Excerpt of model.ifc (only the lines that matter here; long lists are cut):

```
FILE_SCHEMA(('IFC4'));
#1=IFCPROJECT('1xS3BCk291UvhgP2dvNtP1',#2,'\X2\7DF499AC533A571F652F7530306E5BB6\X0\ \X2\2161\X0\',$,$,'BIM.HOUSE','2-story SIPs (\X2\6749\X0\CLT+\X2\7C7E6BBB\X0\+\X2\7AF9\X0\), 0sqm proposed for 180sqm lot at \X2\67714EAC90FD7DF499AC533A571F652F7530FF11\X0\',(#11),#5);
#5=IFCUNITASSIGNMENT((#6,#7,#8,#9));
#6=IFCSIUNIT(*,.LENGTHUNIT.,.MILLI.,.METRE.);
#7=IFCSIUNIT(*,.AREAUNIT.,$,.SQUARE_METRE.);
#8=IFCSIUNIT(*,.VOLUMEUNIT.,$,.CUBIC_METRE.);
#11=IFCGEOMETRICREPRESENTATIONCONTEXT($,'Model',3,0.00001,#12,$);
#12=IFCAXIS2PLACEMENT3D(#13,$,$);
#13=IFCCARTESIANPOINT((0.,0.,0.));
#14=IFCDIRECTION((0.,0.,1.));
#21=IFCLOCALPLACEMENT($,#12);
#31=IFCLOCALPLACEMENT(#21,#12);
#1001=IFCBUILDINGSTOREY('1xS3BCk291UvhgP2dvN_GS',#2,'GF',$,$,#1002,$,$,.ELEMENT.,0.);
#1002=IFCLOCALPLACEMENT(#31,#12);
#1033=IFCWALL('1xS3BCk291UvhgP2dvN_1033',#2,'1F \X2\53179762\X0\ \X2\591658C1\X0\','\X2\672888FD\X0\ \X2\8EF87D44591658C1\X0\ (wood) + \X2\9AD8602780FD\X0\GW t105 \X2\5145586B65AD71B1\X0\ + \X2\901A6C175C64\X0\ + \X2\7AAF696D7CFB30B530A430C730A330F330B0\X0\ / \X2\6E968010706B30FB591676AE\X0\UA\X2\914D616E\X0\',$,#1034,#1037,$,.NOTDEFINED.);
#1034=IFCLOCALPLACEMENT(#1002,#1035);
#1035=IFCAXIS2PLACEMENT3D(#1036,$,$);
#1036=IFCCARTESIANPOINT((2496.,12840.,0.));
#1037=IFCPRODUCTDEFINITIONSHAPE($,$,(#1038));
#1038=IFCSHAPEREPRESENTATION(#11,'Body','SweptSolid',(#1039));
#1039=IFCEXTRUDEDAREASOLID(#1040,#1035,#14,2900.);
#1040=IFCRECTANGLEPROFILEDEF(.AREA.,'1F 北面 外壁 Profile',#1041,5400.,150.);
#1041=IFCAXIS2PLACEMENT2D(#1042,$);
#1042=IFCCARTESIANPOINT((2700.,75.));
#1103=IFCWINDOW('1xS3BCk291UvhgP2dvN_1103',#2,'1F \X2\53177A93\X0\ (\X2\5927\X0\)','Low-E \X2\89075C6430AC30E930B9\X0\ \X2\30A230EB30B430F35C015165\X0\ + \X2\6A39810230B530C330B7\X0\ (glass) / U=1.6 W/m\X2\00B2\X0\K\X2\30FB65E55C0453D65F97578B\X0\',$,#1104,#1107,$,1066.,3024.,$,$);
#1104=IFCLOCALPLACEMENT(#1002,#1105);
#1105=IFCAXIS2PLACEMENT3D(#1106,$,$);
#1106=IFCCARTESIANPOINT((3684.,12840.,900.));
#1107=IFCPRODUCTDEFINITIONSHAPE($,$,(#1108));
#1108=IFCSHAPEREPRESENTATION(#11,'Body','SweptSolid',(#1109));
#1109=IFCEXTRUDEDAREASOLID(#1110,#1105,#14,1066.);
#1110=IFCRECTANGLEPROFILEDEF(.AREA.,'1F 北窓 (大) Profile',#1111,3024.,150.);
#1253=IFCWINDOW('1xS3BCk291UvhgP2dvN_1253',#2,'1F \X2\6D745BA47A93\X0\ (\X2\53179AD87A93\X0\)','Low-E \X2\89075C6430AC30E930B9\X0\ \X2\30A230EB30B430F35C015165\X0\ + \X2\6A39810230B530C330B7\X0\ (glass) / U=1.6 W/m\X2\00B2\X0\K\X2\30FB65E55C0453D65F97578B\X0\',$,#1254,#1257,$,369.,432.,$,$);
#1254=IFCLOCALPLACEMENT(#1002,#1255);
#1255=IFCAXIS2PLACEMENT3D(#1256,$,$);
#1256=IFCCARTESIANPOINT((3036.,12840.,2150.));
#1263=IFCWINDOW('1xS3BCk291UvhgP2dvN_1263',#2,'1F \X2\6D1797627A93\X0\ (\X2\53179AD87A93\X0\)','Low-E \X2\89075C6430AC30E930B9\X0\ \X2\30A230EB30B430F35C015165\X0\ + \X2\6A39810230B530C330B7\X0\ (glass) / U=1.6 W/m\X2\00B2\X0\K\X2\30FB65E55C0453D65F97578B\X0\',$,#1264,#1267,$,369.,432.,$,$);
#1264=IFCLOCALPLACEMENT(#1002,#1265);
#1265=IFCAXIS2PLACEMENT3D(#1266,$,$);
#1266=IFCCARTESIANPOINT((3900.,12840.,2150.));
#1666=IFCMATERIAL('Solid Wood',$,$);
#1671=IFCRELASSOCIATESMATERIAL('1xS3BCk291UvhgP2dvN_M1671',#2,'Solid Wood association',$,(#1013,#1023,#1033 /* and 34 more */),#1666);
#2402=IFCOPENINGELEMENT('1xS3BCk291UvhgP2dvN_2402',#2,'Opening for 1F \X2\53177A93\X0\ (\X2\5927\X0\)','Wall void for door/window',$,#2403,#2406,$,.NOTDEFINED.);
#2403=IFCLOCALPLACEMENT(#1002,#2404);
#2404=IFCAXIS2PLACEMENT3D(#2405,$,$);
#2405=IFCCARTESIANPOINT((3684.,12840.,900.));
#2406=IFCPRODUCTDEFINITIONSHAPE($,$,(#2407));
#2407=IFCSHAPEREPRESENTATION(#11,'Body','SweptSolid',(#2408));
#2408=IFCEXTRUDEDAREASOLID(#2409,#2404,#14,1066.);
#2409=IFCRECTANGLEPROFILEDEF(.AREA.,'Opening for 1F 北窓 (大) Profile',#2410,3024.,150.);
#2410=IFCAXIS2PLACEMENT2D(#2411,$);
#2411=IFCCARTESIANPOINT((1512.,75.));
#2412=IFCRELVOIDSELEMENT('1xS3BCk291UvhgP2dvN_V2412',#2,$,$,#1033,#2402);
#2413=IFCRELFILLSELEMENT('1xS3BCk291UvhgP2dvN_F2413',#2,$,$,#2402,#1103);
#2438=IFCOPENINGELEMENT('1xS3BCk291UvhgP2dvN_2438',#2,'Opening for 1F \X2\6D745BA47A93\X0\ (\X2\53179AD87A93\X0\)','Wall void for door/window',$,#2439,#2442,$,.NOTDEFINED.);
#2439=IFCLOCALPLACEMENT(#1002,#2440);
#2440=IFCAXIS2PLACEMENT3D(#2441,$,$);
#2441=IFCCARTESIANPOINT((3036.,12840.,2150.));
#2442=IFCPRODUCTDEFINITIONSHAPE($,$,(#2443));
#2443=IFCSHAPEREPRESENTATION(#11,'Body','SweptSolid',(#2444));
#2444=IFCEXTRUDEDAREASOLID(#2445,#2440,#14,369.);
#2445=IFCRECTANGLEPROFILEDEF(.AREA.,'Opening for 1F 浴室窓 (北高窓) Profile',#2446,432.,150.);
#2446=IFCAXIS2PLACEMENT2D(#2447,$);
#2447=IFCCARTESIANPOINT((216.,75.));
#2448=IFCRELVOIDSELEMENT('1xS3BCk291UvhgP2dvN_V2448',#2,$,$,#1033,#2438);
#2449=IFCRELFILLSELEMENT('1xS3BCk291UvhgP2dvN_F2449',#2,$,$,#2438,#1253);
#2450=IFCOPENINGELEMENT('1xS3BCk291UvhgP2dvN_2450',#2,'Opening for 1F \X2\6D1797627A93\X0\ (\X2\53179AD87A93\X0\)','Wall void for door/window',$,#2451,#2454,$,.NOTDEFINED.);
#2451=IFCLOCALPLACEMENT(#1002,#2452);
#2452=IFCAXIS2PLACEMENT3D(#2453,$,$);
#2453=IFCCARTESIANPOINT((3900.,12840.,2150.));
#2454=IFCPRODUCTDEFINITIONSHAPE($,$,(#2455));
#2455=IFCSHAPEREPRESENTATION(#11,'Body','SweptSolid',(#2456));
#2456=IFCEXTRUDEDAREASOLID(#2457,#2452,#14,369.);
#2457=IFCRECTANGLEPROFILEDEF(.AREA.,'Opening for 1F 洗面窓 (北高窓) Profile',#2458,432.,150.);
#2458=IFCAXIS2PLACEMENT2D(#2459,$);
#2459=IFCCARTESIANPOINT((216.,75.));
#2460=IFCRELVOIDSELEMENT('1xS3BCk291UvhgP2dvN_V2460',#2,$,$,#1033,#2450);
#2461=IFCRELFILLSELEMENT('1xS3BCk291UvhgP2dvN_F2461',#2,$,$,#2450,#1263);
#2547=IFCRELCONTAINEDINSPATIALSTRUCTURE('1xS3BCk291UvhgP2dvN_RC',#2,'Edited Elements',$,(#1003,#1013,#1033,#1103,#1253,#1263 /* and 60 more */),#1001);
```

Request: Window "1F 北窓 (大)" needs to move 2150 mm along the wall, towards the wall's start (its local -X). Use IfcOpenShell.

```python
import ifcopenshell
import ifcopenshell.api.geometry
import ifcopenshell.util.placement
import ifcopenshell.util.unit

model = ifcopenshell.open("model.ifc")
unit_scale = ifcopenshell.util.unit.calculate_unit_scale(model)

window = model.by_guid("1xS3BCk291UvhgP2dvN_1103")
opening = window.FillsVoids[0].RelatingOpeningElement
wall = opening.VoidsElements[0].RelatingBuildingElement

wall_matrix = ifcopenshell.util.placement.get_local_placement(wall.ObjectPlacement)
shift = wall_matrix[:3, 0] * -2.15 / unit_scale
before = ifcopenshell.util.placement.get_local_placement(window.ObjectPlacement)[:3, 3].copy()

# The window is not placed relative to its opening, so move both.
for product in (opening, window):
    matrix = ifcopenshell.util.placement.get_local_placement(product.ObjectPlacement)
    matrix[:3, 3] += shift
    ifcopenshell.api.geometry.edit_object_placement(model, product=product, matrix=matrix, is_si=False)

after = ifcopenshell.util.placement.get_local_placement(window.ObjectPlacement)[:3, 3]
print("window moved by", (after - before).round(3) + 0.0)

model.write("model_rev.ifc")
```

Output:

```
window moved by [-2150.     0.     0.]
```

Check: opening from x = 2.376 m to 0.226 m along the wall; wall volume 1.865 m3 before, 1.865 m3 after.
